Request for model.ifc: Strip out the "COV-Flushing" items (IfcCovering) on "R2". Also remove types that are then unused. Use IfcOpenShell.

First a look at what the model holds.

```python
import ifcopenshell
import ifcopenshell.util.element

model = ifcopenshell.open("model.ifc")
print(model.schema)
storey = next(s for s in model.by_type("IfcBuildingStorey") if s.Name == "R2")
coverings = [e for e in ifcopenshell.util.element.get_decomposition(storey) if e.is_a("IfcCovering")]
seen = {}
for e in coverings:
    element_type = ifcopenshell.util.element.get_type(e)
    name = element_type.Name if element_type not in (None, e) else None
    seen[name] = seen.get(name, 0) + 1
for name, count in sorted(seen.items(), key=str):
    print(count, "x", name)
```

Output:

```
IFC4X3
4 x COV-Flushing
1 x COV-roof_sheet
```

```python
import ifcopenshell
import ifcopenshell.api.root
import ifcopenshell.util.element

model = ifcopenshell.open("model.ifc")

storey = next(s for s in model.by_type("IfcBuildingStorey") if s.Name == "R2")
coverings = [e for e in ifcopenshell.util.element.get_decomposition(storey) if e.is_a("IfcCovering")]
targets = [e for e in coverings if (t := ifcopenshell.util.element.get_type(e)) not in (None, e) and t.Name == "COV-Flushing"]
types = {ifcopenshell.util.element.get_type(e) for e in targets} - {None, *targets}

for e in targets:
    ifcopenshell.api.root.remove_product(model, product=e)
print(len(targets), "removed")

unused = [t for t in types if not ifcopenshell.util.element.get_types(t)]
for t in unused:
    ifcopenshell.api.root.remove_product(model, product=t)
print(len(unused), "unused types removed")

model.write("model_updated.ifc")
```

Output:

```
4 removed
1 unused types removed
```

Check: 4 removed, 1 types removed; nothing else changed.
